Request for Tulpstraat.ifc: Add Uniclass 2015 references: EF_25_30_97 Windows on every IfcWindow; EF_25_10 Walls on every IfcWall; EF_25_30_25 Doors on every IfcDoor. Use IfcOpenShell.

First a look at what the model holds.

```python
import ifcopenshell

model = ifcopenshell.open("Tulpstraat.ifc")
print(model.schema)
print("classifications:", [c.Name for c in model.by_type("IfcClassification")])
for ifc_class in ("IfcDoor", "IfcRoof", "IfcStair", "IfcWall", "IfcWindow"):
    print(ifc_class, len(model.by_type(ifc_class)))
```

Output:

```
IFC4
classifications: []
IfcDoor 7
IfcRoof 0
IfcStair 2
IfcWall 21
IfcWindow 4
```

```python
import ifcopenshell
import ifcopenshell.api.classification

model = ifcopenshell.open("Tulpstraat.ifc")

system = ifcopenshell.api.classification.add_classification(model, classification="Uniclass 2015")

codes = {
    "IfcWindow": ("EF_25_30_97", "Windows"),
    "IfcWall": ("EF_25_10", "Walls"),
    "IfcDoor": ("EF_25_30_25", "Doors"),
}
for ifc_class, (code, name) in codes.items():
    products = model.by_type(ifc_class)
    ifcopenshell.api.classification.add_reference(
        model, products=products, classification=system, identification=code, name=name
    )
    print(code, len(products))

model.write("Tulpstraat_v2.ifc")
```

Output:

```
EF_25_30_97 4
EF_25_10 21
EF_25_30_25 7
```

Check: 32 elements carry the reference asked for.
